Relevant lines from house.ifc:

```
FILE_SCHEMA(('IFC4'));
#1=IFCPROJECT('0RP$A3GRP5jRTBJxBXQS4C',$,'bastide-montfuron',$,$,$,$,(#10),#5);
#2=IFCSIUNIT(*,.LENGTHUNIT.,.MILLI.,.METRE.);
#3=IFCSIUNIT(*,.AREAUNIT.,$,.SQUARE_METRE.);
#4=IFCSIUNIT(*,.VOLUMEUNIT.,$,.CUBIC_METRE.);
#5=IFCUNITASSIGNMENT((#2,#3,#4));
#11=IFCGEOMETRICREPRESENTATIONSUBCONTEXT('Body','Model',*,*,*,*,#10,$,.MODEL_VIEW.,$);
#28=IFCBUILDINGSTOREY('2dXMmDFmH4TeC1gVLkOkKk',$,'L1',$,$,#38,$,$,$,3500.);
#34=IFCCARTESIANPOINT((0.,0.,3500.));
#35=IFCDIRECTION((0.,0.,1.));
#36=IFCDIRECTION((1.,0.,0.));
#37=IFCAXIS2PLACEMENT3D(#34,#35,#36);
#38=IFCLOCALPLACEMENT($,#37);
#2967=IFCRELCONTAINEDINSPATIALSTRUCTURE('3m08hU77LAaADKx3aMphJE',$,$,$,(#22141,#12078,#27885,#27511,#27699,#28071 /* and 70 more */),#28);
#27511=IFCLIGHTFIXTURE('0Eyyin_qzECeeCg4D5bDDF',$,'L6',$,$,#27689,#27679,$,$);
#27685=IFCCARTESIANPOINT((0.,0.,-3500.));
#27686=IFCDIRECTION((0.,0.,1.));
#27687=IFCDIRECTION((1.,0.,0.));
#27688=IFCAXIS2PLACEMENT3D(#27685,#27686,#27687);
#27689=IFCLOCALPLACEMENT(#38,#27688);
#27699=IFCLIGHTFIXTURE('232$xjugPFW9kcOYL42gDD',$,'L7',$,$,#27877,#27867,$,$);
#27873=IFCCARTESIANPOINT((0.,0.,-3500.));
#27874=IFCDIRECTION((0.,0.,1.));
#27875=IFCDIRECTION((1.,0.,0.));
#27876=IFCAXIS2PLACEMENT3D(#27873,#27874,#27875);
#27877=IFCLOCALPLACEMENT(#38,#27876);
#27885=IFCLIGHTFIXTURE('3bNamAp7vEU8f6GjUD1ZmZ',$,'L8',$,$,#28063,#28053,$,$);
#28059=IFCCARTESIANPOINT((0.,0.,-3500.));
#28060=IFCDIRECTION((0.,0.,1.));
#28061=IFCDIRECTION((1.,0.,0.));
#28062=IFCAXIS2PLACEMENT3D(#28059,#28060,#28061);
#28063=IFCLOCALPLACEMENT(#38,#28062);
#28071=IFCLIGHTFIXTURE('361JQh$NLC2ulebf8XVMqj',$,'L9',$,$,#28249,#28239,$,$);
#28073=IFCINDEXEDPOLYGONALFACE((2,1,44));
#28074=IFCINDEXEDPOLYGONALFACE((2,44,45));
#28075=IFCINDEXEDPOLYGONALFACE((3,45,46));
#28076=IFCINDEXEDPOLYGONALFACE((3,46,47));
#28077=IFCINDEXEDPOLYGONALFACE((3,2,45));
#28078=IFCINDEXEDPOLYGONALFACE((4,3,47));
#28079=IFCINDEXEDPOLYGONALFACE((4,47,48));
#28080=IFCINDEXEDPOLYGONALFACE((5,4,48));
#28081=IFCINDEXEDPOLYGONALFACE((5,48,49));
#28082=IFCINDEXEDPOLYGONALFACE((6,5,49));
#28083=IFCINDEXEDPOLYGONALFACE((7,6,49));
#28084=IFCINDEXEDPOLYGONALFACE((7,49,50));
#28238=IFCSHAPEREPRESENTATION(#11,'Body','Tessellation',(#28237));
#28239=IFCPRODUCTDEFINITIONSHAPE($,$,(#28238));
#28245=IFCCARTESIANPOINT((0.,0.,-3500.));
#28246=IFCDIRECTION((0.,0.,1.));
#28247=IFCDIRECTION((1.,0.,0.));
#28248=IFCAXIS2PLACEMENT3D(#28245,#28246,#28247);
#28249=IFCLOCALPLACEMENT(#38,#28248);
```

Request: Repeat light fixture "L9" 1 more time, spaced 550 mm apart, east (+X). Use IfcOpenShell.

```python
import numpy as np
import ifcopenshell
import ifcopenshell.api.geometry
import ifcopenshell.api.root
import ifcopenshell.util.element
import ifcopenshell.util.placement
import ifcopenshell.util.unit

model = ifcopenshell.open("house.ifc")
unit_scale = ifcopenshell.util.unit.calculate_unit_scale(model)

source = model.by_guid("361JQh$NLC2ulebf8XVMqj")
base = ifcopenshell.util.placement.get_local_placement(source.ObjectPlacement)
step = np.array([1.0, 0.0, 0.0]) * 0.55 / unit_scale

for i in range(1, 2):
    copy = ifcopenshell.api.root.copy_class(model, product=source)
    copy.Representation = ifcopenshell.util.element.copy_deep(
        model, source.Representation, exclude=["IfcGeometricRepresentationContext", "IfcRepresentationMap"]
    )
    matrix = base.copy()
    matrix[:3, 3] += i * step
    print("added at", matrix[:3, 3].round(3) + 0.0)
    ifcopenshell.api.geometry.edit_object_placement(model, product=copy, matrix=matrix, is_si=False)

model.write("house_edited.ifc")
```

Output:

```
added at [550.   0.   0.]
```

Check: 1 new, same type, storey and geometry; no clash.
